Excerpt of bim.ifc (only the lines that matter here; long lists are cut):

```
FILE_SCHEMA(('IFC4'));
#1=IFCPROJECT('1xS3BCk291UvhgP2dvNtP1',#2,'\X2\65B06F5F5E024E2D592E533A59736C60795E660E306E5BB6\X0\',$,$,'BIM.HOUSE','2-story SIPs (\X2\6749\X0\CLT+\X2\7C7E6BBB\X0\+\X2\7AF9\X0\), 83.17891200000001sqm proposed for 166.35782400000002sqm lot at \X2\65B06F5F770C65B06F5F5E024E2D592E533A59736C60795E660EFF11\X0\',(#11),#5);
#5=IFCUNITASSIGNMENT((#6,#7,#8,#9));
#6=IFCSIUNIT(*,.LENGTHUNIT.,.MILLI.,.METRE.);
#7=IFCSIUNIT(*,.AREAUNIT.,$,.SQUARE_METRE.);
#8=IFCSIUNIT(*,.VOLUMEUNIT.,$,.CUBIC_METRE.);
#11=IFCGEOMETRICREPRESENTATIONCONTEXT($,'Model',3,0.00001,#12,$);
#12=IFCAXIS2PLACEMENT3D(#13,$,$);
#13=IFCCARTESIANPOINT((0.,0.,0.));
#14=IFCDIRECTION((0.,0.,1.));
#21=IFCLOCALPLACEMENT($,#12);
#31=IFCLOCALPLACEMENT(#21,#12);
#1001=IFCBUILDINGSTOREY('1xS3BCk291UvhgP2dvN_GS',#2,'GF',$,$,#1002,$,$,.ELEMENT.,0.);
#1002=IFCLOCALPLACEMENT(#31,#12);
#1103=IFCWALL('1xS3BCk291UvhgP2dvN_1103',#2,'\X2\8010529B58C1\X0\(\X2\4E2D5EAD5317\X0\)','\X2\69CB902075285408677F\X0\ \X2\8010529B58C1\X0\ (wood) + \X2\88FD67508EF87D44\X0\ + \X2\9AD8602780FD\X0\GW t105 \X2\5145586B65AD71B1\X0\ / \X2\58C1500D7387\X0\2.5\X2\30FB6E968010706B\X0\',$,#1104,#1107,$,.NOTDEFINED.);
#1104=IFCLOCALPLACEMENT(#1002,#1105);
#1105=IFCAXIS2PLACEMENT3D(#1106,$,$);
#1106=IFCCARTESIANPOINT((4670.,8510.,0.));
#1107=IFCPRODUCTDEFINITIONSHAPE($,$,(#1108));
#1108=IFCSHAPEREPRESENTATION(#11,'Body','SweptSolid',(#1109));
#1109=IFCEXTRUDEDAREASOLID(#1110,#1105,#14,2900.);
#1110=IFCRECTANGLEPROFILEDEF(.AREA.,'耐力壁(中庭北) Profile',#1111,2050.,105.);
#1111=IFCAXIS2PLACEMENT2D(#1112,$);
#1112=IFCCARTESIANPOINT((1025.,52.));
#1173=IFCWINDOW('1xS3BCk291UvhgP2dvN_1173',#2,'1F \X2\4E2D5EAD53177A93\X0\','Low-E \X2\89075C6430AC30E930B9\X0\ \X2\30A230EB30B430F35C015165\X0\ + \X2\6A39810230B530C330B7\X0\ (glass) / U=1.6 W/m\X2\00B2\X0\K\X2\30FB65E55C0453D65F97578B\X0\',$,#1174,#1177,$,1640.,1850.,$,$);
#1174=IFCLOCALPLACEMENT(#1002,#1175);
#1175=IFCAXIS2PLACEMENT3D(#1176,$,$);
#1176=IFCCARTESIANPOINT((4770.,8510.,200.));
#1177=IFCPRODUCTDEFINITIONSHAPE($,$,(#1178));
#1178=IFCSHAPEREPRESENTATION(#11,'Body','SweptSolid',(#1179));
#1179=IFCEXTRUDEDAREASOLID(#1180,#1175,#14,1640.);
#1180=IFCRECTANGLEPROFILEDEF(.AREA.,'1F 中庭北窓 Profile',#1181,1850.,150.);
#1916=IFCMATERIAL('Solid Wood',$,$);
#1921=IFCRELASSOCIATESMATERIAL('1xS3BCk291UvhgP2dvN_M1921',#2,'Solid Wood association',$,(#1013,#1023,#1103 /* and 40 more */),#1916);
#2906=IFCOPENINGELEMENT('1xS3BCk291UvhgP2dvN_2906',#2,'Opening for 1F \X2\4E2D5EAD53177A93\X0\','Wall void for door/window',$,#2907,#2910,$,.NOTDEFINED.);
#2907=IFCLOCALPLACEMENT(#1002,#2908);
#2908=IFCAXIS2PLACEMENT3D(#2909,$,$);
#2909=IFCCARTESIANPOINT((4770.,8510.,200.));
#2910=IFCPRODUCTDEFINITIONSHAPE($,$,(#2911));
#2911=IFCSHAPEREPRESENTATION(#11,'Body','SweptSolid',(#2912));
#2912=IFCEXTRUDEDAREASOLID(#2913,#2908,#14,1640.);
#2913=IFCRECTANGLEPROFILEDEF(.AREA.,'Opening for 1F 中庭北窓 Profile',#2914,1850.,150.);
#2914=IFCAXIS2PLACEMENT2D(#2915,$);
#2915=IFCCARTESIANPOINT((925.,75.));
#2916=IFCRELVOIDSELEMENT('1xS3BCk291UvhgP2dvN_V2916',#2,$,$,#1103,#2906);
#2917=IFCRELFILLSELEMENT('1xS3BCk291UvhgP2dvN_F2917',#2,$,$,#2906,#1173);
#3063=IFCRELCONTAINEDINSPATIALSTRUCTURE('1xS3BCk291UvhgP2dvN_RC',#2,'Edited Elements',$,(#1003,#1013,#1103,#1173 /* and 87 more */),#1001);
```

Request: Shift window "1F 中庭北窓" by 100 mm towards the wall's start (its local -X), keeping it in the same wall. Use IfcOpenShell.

```python
import ifcopenshell
import ifcopenshell.api.geometry
import ifcopenshell.util.placement
import ifcopenshell.util.unit

model = ifcopenshell.open("bim.ifc")
unit_scale = ifcopenshell.util.unit.calculate_unit_scale(model)

window = model.by_guid("1xS3BCk291UvhgP2dvN_1173")
opening = window.FillsVoids[0].RelatingOpeningElement
wall = opening.VoidsElements[0].RelatingBuildingElement

wall_matrix = ifcopenshell.util.placement.get_local_placement(wall.ObjectPlacement)
shift = wall_matrix[:3, 0] * -0.1 / unit_scale
before = ifcopenshell.util.placement.get_local_placement(window.ObjectPlacement)[:3, 3].copy()

# The window is not placed relative to its opening, so move both.
for product in (opening, window):
    matrix = ifcopenshell.util.placement.get_local_placement(product.ObjectPlacement)
    matrix[:3, 3] += shift
    ifcopenshell.api.geometry.edit_object_placement(model, product=product, matrix=matrix, is_si=False)

after = ifcopenshell.util.placement.get_local_placement(window.ObjectPlacement)[:3, 3]
print("window moved by", (after - before).round(3) + 0.0)

model.write("bim_edited.ifc")
```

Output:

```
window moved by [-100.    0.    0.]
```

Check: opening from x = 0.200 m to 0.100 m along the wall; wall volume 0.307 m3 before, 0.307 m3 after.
